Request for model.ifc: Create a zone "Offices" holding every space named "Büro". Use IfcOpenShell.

First a look at what the model holds.

```python
import ifcopenshell

model = ifcopenshell.open("model.ifc")
print(model.schema)
seen = {}
for space in model.by_type("IfcSpace"):
    seen[space.LongName] = seen.get(space.LongName, 0) + 1
for name, count in sorted(seen.items(), key=str):
    print(count, "x", name)
print("zones:", [z.Name for z in model.by_type("IfcZone")][:20])
```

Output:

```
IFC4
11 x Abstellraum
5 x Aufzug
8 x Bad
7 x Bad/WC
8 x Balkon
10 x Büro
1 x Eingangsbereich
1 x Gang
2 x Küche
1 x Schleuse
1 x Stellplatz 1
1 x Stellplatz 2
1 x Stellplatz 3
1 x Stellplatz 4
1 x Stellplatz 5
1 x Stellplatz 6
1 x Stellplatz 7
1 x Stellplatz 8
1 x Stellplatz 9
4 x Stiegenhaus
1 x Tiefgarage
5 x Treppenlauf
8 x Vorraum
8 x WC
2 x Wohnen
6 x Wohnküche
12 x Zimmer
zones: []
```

```python
import ifcopenshell
import ifcopenshell.api.group
import ifcopenshell.api.root

model = ifcopenshell.open("model.ifc")

names = {"Büro"}
spaces = [s for s in model.by_type("IfcSpace") if s.LongName in names]

zone = ifcopenshell.api.root.create_entity(model, ifc_class="IfcZone", name="Offices")
ifcopenshell.api.group.assign_group(model, products=spaces, group=zone)
print(len(spaces), "spaces in", zone.Name)

model.write("model-out.ifc")
```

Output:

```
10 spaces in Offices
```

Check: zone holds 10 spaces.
